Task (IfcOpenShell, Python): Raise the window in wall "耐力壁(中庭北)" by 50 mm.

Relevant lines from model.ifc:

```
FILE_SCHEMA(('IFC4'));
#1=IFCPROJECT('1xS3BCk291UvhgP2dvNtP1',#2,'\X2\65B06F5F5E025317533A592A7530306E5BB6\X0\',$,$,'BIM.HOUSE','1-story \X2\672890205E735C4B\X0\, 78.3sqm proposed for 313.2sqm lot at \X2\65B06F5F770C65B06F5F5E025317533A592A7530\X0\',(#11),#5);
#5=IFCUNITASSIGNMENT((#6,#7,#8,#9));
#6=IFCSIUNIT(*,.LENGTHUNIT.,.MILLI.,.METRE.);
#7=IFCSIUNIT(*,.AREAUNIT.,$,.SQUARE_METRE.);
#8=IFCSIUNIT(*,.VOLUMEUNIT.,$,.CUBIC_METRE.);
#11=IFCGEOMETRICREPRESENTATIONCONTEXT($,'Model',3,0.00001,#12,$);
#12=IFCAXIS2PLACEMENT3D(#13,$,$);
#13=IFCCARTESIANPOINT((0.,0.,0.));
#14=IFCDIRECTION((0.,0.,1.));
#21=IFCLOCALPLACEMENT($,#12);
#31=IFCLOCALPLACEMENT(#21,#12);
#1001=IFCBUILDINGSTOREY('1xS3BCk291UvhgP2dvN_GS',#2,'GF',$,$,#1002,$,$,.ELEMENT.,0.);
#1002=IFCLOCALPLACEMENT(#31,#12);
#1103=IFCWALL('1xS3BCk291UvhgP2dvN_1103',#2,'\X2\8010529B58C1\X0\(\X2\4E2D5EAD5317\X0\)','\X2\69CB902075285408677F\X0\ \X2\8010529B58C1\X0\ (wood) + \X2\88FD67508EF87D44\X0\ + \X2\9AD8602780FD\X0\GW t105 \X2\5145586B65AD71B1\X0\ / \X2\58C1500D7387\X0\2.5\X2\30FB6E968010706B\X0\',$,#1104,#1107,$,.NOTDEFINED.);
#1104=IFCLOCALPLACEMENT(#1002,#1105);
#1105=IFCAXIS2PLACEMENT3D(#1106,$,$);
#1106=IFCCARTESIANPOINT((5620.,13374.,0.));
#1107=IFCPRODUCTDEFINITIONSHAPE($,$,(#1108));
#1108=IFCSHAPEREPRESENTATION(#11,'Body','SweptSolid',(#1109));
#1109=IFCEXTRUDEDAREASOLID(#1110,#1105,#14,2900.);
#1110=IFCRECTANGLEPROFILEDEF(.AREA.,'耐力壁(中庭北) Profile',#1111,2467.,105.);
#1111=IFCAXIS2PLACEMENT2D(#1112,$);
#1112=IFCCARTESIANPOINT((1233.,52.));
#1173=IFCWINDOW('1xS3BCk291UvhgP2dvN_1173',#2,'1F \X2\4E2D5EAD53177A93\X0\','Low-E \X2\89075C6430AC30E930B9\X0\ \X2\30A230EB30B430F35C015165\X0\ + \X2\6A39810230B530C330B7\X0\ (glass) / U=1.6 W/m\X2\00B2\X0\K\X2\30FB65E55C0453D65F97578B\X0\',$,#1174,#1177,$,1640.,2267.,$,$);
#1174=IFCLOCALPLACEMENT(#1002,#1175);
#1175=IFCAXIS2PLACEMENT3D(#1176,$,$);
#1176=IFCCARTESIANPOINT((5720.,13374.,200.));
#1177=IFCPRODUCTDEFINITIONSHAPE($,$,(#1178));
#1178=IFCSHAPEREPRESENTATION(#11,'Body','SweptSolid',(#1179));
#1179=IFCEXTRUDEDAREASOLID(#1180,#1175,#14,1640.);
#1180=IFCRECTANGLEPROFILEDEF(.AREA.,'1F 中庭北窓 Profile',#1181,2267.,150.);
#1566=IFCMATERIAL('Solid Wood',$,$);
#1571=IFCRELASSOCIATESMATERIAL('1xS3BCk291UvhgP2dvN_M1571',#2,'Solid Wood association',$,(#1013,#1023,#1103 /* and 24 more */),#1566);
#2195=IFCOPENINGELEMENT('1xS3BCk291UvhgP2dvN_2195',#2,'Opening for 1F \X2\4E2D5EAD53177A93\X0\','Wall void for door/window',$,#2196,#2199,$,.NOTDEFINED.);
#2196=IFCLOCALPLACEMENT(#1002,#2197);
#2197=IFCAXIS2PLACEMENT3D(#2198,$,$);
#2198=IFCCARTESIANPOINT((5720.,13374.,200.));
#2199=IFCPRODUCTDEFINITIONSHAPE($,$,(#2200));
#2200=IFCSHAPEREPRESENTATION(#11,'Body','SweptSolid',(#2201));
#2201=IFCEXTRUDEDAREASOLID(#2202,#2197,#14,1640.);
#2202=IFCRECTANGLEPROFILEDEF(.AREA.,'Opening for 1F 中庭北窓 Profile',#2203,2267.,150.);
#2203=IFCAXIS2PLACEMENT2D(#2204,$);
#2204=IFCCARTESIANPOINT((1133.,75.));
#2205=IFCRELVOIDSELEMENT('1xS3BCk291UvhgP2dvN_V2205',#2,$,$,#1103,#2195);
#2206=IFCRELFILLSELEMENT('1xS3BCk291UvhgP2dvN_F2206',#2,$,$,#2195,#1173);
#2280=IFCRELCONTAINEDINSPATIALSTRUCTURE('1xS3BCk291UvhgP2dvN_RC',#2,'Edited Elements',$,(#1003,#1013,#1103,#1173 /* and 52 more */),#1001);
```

```python
import numpy as np
import ifcopenshell
import ifcopenshell.api.geometry
import ifcopenshell.util.placement
import ifcopenshell.util.unit

model = ifcopenshell.open("model.ifc")
unit_scale = ifcopenshell.util.unit.calculate_unit_scale(model)

window = model.by_id(1173)
opening = window.FillsVoids[0].RelatingOpeningElement
dz = 0.05 / unit_scale

shift = np.array([0.0, 0.0, dz])
# The window is not placed relative to its opening, so move both.
for product in (opening, window):
    matrix = ifcopenshell.util.placement.get_local_placement(product.ObjectPlacement)
    matrix[:3, 3] += shift
    ifcopenshell.api.geometry.edit_object_placement(model, product=product, matrix=matrix, is_si=False)

print(f"moved by {dz * unit_scale:+.3f} m")

model.write("model_v2.ifc")
```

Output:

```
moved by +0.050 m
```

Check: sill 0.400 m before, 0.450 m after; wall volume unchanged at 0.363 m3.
